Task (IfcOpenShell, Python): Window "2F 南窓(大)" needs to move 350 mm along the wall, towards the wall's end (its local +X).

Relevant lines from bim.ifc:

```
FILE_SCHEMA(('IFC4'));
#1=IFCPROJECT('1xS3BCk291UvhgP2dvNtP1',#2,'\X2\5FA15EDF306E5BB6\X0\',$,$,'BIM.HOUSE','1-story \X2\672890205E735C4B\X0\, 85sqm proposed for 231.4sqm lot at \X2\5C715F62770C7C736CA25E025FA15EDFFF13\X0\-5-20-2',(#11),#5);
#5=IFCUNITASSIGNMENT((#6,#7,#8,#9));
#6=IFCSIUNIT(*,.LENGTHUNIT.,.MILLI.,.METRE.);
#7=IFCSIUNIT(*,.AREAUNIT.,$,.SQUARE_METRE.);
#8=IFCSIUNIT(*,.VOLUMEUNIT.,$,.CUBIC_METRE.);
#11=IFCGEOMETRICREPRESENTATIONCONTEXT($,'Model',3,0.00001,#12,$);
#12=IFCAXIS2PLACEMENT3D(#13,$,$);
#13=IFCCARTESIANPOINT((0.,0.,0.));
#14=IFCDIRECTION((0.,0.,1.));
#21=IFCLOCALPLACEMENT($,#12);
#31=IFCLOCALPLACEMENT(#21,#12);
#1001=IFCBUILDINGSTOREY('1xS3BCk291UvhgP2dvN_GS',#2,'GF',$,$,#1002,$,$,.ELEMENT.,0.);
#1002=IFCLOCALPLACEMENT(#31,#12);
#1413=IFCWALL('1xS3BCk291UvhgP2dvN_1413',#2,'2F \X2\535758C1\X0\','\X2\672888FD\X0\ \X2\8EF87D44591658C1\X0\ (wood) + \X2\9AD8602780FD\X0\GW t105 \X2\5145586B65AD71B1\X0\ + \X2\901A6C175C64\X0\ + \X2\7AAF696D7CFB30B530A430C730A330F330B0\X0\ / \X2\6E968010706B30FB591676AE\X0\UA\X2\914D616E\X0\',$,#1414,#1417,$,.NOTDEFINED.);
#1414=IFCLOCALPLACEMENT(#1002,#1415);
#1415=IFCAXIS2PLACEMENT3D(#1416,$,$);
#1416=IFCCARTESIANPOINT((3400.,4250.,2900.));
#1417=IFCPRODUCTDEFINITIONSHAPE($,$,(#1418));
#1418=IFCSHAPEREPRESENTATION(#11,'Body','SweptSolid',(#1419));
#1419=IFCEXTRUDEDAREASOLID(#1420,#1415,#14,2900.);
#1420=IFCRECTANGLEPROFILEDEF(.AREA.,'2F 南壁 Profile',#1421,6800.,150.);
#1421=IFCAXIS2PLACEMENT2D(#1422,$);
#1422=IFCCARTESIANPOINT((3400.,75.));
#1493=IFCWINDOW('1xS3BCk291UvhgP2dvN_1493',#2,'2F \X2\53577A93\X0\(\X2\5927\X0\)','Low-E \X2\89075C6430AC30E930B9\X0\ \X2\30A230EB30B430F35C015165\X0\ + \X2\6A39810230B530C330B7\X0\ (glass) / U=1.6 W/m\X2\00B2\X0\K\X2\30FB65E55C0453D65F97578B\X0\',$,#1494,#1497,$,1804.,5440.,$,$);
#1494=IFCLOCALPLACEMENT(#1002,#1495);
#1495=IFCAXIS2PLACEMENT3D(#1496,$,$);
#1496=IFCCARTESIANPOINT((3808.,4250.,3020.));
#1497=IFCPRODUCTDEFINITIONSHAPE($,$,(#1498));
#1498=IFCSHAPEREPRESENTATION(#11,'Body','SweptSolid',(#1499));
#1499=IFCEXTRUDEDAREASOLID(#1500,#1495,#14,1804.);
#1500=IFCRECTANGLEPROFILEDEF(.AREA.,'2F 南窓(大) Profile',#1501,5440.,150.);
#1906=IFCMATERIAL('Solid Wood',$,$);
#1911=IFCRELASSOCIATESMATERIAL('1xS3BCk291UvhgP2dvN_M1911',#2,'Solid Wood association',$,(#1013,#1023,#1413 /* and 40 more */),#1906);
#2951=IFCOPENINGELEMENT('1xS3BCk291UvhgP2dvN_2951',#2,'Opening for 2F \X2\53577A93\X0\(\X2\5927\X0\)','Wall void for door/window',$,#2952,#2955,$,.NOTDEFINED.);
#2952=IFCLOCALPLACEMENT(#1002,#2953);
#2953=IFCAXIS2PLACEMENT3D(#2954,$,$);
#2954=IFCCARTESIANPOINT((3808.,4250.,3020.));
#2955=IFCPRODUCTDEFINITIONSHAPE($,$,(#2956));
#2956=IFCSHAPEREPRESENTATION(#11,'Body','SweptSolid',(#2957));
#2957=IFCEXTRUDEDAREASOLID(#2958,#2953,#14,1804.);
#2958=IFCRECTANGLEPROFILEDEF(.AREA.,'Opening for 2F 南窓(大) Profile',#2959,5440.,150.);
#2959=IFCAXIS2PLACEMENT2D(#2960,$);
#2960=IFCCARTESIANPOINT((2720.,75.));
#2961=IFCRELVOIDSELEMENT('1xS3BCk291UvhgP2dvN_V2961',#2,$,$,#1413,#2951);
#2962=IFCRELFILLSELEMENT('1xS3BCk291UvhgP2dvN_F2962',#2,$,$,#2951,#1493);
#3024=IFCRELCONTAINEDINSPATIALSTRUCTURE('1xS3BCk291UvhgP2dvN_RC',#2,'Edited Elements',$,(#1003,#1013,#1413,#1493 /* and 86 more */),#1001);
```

```python
import ifcopenshell
import ifcopenshell.api.geometry
import ifcopenshell.util.placement

model = ifcopenshell.open("bim.ifc")

window = model.by_guid("1xS3BCk291UvhgP2dvN_1493")
opening = window.FillsVoids[0].RelatingOpeningElement
wall = opening.VoidsElements[0].RelatingBuildingElement

wall_matrix = ifcopenshell.util.placement.get_local_placement(wall.ObjectPlacement)
shift = wall_matrix[:3, 0] * 350.0
before = ifcopenshell.util.placement.get_local_placement(window.ObjectPlacement)[:3, 3].copy()

# The window is not placed relative to its opening, so move both.
for product in (opening, window):
    matrix = ifcopenshell.util.placement.get_local_placement(product.ObjectPlacement)
    matrix[:3, 3] += shift
    ifcopenshell.api.geometry.edit_object_placement(model, product=product, matrix=matrix, is_si=False)

after = ifcopenshell.util.placement.get_local_placement(window.ObjectPlacement)[:3, 3]
print("window moved by", (after - before).round(3) + 0.0)

model.write("bim-out.ifc")
```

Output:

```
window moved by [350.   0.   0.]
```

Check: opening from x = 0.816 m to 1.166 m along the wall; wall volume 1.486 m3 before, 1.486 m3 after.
